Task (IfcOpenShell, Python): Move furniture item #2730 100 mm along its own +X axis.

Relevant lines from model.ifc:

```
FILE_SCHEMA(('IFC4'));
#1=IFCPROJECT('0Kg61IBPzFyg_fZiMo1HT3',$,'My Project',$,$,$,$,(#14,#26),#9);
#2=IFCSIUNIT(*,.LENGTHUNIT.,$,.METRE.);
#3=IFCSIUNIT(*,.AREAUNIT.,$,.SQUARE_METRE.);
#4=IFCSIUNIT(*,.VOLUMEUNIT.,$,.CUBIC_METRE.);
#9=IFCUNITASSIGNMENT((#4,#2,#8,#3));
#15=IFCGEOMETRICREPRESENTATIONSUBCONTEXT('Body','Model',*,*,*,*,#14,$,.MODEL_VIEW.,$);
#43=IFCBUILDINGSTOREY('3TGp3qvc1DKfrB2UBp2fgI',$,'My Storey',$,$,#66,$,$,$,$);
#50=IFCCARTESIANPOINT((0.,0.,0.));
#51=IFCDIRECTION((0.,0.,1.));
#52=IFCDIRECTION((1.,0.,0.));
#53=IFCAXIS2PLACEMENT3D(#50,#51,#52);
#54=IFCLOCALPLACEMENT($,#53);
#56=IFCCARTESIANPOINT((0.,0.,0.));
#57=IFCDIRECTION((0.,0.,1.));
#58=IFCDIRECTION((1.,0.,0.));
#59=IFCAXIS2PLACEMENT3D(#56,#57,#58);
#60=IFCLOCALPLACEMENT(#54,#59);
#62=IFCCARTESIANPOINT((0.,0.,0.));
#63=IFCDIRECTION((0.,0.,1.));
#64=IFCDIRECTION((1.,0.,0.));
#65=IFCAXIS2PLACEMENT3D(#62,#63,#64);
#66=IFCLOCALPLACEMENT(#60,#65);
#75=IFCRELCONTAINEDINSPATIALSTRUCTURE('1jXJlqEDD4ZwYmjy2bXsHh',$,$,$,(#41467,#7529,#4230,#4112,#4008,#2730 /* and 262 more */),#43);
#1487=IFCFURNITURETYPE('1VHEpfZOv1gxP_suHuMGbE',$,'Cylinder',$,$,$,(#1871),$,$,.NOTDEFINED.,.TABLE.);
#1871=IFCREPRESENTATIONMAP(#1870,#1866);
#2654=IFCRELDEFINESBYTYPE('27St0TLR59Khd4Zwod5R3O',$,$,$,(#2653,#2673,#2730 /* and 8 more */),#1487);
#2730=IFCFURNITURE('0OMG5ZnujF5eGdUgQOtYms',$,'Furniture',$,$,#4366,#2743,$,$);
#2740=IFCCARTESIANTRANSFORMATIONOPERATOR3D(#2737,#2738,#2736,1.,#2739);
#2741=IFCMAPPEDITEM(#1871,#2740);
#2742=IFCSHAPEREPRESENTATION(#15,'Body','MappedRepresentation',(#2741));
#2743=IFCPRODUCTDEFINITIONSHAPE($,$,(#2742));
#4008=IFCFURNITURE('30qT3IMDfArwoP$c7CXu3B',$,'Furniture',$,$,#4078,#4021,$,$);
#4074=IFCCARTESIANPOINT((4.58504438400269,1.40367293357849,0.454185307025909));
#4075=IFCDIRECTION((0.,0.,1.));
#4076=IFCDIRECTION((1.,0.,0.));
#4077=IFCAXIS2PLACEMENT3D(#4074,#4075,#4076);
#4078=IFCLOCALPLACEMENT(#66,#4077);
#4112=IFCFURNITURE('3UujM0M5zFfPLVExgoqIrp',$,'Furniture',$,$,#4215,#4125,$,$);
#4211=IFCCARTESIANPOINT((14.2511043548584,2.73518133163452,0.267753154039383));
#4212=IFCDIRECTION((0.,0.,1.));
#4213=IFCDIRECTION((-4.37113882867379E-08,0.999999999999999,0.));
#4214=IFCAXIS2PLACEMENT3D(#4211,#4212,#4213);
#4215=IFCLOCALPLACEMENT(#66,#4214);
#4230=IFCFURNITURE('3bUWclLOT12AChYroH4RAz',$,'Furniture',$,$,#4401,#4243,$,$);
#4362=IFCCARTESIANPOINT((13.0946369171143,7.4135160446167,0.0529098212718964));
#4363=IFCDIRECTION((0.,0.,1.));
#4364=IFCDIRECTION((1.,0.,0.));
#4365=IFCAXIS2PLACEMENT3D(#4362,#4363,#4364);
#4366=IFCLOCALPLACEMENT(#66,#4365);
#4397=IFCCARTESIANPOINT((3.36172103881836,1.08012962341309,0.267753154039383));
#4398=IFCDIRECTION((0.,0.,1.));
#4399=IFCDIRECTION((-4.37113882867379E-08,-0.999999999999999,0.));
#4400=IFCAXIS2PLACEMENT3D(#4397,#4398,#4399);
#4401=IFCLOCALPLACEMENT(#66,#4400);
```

```python
import ifcopenshell
import ifcopenshell.api.geometry
import ifcopenshell.util.placement

model = ifcopenshell.open("model.ifc")

item = model.by_guid("0OMG5ZnujF5eGdUgQOtYms")
matrix = ifcopenshell.util.placement.get_local_placement(item.ObjectPlacement)
matrix[:3, 3] += matrix[:3, 0] * 0.1
ifcopenshell.api.geometry.edit_object_placement(model, product=item, matrix=matrix, is_si=False)

print(ifcopenshell.util.placement.get_local_placement(item.ObjectPlacement).round(3) + 0.0)

model.write("model_rev.ifc")
```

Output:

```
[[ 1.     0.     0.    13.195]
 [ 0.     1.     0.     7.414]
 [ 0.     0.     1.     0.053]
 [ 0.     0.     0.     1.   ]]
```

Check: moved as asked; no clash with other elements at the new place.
